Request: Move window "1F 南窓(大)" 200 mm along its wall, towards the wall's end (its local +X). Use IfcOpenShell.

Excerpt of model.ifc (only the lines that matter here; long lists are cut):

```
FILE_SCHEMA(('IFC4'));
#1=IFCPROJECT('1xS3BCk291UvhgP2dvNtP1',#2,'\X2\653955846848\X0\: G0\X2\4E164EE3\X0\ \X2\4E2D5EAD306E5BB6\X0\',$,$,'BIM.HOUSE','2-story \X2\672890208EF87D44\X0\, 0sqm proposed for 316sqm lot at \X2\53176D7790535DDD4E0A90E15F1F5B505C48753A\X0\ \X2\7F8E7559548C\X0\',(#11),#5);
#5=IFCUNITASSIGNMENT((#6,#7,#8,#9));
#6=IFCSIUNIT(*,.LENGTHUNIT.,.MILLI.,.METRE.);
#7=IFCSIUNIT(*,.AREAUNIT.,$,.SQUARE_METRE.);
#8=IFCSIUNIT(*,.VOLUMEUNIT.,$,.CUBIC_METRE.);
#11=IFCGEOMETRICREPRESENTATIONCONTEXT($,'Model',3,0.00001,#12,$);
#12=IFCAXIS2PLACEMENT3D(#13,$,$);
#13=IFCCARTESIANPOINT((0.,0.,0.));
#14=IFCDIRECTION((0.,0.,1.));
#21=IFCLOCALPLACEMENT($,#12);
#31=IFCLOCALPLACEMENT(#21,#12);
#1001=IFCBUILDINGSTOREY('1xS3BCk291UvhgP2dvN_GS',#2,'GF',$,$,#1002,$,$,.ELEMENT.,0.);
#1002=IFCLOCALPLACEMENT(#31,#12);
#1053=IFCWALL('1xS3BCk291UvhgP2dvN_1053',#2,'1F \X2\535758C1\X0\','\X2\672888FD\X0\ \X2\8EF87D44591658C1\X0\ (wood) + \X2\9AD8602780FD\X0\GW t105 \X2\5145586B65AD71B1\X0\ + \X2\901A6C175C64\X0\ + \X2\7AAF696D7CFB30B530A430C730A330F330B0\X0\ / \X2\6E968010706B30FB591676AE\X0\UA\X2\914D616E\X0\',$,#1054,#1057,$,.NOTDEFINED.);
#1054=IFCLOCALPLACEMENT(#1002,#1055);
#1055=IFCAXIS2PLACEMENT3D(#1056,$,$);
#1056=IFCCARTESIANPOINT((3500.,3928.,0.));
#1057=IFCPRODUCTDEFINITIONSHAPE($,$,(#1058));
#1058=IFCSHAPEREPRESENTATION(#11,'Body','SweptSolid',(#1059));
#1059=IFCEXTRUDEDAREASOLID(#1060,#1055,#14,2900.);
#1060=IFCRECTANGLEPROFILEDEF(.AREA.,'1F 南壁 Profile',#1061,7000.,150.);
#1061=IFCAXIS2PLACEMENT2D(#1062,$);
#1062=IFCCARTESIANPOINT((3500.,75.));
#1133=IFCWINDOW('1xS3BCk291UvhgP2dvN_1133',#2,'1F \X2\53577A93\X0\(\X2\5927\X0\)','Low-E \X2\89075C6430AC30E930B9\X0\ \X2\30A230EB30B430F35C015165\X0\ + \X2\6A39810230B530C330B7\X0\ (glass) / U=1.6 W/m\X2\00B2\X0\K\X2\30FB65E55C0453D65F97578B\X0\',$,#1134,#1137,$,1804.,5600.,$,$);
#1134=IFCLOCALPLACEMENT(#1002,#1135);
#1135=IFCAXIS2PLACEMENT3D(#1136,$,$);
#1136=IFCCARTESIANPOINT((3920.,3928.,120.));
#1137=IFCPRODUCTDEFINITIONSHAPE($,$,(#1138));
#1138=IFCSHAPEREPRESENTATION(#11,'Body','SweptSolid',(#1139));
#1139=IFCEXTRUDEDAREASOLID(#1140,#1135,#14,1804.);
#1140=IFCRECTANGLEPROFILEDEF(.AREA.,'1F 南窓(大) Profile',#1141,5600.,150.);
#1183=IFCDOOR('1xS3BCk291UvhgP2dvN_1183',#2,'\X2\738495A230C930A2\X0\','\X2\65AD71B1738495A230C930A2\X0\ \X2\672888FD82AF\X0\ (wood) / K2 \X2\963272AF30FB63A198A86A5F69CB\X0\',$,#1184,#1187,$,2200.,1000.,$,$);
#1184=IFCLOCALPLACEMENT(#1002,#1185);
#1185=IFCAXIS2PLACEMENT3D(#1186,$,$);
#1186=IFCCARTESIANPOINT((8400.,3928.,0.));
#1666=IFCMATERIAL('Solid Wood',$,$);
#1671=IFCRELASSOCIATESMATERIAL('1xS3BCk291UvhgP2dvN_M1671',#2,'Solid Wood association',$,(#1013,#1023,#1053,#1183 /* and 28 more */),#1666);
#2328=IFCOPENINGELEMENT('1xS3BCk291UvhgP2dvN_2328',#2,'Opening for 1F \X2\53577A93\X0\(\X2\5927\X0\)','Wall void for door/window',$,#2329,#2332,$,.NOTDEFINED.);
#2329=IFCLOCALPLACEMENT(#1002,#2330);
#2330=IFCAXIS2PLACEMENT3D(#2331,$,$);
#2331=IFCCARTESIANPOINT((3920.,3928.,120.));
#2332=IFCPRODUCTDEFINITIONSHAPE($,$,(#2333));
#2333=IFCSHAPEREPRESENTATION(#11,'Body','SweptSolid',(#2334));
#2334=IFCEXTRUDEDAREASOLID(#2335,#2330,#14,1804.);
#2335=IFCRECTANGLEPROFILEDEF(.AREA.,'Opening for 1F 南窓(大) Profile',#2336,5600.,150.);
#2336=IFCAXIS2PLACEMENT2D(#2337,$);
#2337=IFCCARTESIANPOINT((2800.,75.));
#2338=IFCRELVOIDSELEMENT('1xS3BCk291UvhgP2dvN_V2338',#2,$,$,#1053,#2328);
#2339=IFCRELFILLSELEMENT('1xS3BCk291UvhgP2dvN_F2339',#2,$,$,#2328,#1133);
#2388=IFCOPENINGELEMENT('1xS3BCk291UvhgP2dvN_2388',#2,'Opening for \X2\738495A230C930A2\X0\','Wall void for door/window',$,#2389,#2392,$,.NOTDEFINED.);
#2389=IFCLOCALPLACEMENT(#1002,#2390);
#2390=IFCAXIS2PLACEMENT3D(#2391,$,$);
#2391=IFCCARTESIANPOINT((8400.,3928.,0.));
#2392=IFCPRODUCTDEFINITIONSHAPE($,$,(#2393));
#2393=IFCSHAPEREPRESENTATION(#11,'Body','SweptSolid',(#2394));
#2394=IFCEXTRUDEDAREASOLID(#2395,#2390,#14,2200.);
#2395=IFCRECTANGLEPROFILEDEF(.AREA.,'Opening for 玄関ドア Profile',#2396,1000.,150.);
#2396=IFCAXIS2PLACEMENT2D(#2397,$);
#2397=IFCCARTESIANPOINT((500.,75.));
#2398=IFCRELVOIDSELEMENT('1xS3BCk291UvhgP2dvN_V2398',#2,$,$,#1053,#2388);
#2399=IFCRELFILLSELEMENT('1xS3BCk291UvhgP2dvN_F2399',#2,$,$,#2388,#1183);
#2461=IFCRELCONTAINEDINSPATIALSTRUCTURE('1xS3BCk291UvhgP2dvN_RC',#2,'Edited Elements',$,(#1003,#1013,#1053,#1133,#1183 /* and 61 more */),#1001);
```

```python
import ifcopenshell
import ifcopenshell.api.geometry
import ifcopenshell.util.placement
import ifcopenshell.util.unit

model = ifcopenshell.open("model.ifc")
unit_scale = ifcopenshell.util.unit.calculate_unit_scale(model)

window = model.by_guid("1xS3BCk291UvhgP2dvN_1133")
opening = window.FillsVoids[0].RelatingOpeningElement
wall = opening.VoidsElements[0].RelatingBuildingElement

wall_matrix = ifcopenshell.util.placement.get_local_placement(wall.ObjectPlacement)
shift = wall_matrix[:3, 0] * 0.2 / unit_scale
before = ifcopenshell.util.placement.get_local_placement(window.ObjectPlacement)[:3, 3].copy()

# The window is not placed relative to its opening, so move both.
for product in (opening, window):
    matrix = ifcopenshell.util.placement.get_local_placement(product.ObjectPlacement)
    matrix[:3, 3] += shift
    ifcopenshell.api.geometry.edit_object_placement(model, product=product, matrix=matrix, is_si=False)

after = ifcopenshell.util.placement.get_local_placement(window.ObjectPlacement)[:3, 3]
print("window moved by", (after - before).round(3) + 0.0)

model.write("model_edited.ifc")
```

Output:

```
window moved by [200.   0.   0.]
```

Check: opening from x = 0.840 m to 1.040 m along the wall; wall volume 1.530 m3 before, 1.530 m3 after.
